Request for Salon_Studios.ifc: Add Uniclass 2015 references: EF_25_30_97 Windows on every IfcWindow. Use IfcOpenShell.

First a look at what the model holds.

```python
import ifcopenshell

model = ifcopenshell.open("Salon_Studios.ifc")
print(model.schema)
print("classifications:", [c.Name for c in model.by_type("IfcClassification")])
for ifc_class in ("IfcDoor", "IfcRoof", "IfcStair", "IfcWall", "IfcWindow"):
    print(ifc_class, len(model.by_type(ifc_class)))
```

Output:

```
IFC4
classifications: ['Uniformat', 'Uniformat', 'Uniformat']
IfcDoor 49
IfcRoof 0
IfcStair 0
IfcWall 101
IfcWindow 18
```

```python
import ifcopenshell
import ifcopenshell.api.classification

model = ifcopenshell.open("Salon_Studios.ifc")

system = ifcopenshell.api.classification.add_classification(model, classification="Uniclass 2015")

codes = {
    "IfcWindow": ("EF_25_30_97", "Windows"),
}
for ifc_class, (code, name) in codes.items():
    products = model.by_type(ifc_class)
    ifcopenshell.api.classification.add_reference(
        model, products=products, classification=system, identification=code, name=name
    )
    print(code, len(products))

model.write("Salon_Studios_rev.ifc")
```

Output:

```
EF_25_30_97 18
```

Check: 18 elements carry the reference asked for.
